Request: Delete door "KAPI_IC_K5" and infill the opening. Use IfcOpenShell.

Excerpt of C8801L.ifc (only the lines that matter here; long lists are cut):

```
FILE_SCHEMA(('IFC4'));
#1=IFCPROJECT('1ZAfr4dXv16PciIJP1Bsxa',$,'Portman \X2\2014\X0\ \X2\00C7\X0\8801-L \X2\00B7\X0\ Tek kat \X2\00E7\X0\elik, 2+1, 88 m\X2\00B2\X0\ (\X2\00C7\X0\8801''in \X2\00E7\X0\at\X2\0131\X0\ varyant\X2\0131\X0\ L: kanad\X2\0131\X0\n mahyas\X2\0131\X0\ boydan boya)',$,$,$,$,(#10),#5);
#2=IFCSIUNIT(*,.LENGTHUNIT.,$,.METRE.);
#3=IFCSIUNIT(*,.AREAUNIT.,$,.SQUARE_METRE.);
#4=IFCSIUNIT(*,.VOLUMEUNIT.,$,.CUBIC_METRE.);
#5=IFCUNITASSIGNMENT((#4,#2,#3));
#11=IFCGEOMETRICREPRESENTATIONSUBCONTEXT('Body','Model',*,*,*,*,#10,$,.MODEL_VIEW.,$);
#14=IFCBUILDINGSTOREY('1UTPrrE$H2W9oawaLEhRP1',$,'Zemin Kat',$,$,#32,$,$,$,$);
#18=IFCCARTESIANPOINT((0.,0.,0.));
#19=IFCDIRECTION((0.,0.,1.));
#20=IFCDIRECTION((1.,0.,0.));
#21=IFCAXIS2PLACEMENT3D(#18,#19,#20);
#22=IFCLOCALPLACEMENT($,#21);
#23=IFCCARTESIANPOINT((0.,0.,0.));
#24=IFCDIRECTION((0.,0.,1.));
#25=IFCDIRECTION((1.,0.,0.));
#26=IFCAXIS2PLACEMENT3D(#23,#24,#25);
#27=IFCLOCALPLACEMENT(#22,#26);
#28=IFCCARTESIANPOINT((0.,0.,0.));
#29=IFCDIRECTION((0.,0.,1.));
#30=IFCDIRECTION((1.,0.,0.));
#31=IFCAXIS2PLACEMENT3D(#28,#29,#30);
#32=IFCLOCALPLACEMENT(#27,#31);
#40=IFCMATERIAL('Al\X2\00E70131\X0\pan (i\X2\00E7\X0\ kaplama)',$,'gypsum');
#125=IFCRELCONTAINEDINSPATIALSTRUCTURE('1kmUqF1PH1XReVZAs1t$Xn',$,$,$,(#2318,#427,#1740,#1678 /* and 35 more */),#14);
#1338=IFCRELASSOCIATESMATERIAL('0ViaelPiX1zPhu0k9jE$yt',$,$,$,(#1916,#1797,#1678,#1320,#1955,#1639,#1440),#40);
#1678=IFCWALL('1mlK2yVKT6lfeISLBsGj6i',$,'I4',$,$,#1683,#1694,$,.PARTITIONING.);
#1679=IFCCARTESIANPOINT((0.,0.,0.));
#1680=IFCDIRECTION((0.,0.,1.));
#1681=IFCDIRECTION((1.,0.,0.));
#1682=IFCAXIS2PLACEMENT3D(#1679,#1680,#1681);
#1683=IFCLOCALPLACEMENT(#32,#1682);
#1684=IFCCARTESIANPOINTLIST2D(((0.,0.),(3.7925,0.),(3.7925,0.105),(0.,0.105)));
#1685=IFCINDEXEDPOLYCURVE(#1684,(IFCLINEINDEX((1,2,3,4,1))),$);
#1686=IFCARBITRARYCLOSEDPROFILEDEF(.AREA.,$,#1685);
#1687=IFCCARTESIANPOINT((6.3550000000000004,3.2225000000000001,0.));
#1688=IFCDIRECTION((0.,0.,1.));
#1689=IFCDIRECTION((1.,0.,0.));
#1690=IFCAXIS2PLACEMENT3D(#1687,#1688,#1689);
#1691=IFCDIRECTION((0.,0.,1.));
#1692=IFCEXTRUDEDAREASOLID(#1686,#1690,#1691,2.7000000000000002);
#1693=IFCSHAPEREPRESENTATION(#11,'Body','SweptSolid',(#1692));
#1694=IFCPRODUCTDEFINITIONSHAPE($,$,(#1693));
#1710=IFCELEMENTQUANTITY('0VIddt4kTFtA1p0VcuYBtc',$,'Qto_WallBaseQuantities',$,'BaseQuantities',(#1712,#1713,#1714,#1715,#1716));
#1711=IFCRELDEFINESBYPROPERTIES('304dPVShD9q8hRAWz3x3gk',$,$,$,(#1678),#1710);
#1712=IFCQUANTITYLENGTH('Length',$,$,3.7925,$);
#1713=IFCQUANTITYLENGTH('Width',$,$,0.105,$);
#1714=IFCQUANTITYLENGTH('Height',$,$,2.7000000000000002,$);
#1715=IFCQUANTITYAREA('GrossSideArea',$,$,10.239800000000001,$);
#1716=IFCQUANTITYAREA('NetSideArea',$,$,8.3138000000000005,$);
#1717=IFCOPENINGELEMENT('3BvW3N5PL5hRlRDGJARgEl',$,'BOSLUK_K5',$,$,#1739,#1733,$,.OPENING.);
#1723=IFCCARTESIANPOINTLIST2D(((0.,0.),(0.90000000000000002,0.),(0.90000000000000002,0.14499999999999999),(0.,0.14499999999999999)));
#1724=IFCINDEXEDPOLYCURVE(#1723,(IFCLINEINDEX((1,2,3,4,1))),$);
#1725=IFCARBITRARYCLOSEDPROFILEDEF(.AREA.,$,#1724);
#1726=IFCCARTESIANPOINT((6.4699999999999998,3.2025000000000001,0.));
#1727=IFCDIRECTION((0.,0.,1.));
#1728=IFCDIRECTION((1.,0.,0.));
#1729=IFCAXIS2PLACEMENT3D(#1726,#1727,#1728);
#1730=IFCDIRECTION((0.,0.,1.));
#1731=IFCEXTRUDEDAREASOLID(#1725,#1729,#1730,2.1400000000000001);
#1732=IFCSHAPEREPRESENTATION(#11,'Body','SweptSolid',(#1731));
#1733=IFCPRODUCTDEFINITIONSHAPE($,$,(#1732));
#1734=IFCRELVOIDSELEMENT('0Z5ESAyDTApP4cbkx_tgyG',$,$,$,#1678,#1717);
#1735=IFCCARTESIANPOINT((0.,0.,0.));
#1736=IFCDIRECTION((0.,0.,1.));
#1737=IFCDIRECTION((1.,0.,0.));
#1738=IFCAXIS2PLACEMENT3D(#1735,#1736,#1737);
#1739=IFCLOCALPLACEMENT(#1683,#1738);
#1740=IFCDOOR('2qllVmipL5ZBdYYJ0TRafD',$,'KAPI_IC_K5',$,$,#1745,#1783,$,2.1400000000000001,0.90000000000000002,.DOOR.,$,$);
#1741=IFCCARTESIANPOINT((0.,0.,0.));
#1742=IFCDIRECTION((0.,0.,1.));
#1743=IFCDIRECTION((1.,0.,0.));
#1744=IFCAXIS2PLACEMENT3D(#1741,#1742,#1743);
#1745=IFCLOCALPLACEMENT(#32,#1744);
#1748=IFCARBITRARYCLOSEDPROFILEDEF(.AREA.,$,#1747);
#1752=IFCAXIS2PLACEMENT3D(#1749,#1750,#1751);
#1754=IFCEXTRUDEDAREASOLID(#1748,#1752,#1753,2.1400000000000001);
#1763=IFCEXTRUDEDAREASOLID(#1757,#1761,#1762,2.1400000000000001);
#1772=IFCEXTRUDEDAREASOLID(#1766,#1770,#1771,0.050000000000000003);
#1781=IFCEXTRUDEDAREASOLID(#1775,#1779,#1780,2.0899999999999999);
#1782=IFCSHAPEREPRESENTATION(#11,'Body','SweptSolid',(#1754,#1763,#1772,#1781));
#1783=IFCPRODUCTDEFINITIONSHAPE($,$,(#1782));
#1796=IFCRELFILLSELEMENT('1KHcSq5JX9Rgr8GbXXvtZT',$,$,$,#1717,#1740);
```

```python
import ifcopenshell
import ifcopenshell.api.feature
import ifcopenshell.api.pset
import ifcopenshell.api.root
import ifcopenshell.geom
import ifcopenshell.util.element
import ifcopenshell.util.shape
import ifcopenshell.util.unit

model = ifcopenshell.open("C8801L.ifc")
area_scale = ifcopenshell.util.unit.calculate_unit_scale(model, "AREAUNIT")
settings = ifcopenshell.geom.settings()


def volume(element):
    """Net volume in cubic metres, openings subtracted."""
    shape = ifcopenshell.geom.create_shape(settings, element)
    return ifcopenshell.util.shape.get_volume(shape.geometry)


door = model.by_guid("2qllVmipL5ZBdYYJ0TRafD")
opening = door.FillsVoids[0].RelatingOpeningElement
wall = opening.VoidsElements[0].RelatingBuildingElement
before = volume(wall)

ifcopenshell.api.root.remove_product(model, product=door)
ifcopenshell.api.feature.remove_feature(model, feature=opening)

after = volume(wall)
thickness = 0.105  # wall thickness in metres

# Update the wall's stored quantities.
qto = model.by_id(ifcopenshell.util.element.get_pset(wall, "Qto_WallBaseQuantities", should_inherit=False)["id"])
ifcopenshell.api.pset.edit_qto(model, qto=qto, properties={"NetSideArea": after / thickness / area_scale})

print(f"wall volume {before:.3f} -> {after:.3f} m3")

model.write("C8801L-out.ifc")
```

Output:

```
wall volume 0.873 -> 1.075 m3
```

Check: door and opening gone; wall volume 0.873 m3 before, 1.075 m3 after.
